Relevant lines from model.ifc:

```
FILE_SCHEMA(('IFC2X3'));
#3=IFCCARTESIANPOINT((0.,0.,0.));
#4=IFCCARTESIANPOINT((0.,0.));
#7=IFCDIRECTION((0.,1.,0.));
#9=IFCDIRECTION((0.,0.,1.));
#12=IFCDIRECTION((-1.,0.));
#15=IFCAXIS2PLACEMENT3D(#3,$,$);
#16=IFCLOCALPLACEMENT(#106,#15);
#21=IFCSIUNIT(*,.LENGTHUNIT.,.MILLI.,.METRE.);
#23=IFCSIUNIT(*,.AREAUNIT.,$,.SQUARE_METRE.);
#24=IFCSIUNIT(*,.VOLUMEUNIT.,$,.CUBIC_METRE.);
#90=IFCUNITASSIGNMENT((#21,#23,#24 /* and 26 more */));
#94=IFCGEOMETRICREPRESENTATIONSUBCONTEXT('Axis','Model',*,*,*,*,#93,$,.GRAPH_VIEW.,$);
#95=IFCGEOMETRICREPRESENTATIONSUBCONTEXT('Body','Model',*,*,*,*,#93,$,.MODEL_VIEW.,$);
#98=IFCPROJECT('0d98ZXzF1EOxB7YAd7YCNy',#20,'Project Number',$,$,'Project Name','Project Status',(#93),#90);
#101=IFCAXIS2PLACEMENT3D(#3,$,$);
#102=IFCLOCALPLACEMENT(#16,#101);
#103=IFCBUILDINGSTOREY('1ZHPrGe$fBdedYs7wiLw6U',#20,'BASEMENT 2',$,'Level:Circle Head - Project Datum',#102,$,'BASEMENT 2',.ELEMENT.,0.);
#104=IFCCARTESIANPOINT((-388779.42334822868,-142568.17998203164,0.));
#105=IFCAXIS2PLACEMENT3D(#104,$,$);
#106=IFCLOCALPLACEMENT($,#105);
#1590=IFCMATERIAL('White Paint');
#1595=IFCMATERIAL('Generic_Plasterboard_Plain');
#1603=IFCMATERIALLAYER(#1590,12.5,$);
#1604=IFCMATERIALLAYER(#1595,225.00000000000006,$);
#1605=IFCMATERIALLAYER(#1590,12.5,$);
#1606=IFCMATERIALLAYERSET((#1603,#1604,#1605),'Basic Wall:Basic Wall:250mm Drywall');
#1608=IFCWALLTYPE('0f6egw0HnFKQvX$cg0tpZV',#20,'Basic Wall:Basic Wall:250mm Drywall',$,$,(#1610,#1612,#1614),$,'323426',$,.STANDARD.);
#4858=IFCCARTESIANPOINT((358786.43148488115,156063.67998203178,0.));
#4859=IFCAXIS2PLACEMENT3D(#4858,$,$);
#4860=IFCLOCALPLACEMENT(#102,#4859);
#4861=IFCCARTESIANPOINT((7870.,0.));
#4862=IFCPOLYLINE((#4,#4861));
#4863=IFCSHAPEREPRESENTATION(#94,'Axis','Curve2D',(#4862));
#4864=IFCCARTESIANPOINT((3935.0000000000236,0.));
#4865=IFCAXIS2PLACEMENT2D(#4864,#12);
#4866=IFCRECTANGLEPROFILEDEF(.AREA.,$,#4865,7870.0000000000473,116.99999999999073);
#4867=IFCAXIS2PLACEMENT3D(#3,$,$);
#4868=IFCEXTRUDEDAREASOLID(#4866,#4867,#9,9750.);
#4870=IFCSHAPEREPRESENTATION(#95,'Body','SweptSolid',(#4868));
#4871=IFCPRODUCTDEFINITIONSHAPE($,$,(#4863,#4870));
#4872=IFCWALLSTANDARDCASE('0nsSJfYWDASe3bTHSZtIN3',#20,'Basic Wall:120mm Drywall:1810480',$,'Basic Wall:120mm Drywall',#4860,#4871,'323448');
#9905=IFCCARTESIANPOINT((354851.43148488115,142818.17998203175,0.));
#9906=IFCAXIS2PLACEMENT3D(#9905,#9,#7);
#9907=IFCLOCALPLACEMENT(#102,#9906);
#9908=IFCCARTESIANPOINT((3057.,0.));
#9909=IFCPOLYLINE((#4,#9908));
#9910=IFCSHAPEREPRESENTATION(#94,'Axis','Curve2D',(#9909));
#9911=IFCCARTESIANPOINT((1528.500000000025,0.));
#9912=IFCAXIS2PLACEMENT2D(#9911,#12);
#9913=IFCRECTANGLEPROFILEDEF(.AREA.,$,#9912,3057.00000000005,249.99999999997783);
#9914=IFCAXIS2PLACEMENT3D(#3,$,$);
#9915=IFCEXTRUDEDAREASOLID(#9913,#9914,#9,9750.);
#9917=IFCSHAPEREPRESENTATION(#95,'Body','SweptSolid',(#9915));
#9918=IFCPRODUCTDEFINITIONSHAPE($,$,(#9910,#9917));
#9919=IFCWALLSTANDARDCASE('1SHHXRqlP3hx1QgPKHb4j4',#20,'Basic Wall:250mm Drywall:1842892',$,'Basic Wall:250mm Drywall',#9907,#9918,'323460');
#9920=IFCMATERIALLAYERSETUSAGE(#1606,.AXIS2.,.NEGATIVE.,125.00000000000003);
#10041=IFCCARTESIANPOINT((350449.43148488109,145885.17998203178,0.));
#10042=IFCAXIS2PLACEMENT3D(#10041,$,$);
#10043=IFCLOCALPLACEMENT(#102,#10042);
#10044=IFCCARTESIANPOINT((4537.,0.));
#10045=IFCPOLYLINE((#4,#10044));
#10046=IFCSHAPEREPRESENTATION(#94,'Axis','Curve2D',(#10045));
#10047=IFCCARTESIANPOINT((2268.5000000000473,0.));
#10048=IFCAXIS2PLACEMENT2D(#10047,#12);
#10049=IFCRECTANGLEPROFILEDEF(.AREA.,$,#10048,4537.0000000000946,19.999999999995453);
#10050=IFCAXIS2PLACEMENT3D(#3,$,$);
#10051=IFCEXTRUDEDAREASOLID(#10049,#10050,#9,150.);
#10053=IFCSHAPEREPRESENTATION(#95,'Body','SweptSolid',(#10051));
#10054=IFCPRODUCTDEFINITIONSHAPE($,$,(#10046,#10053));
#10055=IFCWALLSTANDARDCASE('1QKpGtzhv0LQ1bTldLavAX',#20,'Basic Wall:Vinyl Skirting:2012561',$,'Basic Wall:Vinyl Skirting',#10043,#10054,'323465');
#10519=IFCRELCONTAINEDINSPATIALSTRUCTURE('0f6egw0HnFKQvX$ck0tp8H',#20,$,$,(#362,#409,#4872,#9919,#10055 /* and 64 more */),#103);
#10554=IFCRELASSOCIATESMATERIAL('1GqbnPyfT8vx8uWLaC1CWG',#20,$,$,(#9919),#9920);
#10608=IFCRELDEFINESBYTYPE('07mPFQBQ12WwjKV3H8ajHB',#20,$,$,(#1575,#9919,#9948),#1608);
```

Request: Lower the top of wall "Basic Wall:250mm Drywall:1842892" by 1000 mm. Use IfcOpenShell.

```python
import ifcopenshell
import ifcopenshell.geom
import ifcopenshell.util.representation
import ifcopenshell.util.shape

model = ifcopenshell.open("model.ifc")
settings = ifcopenshell.geom.settings()


def volume(element):
    """Net volume in cubic metres, openings subtracted."""
    shape = ifcopenshell.geom.create_shape(settings, element)
    return ifcopenshell.util.shape.get_volume(shape.geometry)


wall = model.by_guid("1SHHXRqlP3hx1QgPKHb4j4")
before = volume(wall)

body = ifcopenshell.util.representation.get_representation(wall, "Model", "Body")
solid = body.Items[0]
old_height = solid.Depth
solid.Depth -= 1000.0
after = volume(wall)

print(f"height {old_height:g} -> {solid.Depth:g}, volume {before:.3f} -> {after:.3f} m3")

model.write("model_rev.ifc")
```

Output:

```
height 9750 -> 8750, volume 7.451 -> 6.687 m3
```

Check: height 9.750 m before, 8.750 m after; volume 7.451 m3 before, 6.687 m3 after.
